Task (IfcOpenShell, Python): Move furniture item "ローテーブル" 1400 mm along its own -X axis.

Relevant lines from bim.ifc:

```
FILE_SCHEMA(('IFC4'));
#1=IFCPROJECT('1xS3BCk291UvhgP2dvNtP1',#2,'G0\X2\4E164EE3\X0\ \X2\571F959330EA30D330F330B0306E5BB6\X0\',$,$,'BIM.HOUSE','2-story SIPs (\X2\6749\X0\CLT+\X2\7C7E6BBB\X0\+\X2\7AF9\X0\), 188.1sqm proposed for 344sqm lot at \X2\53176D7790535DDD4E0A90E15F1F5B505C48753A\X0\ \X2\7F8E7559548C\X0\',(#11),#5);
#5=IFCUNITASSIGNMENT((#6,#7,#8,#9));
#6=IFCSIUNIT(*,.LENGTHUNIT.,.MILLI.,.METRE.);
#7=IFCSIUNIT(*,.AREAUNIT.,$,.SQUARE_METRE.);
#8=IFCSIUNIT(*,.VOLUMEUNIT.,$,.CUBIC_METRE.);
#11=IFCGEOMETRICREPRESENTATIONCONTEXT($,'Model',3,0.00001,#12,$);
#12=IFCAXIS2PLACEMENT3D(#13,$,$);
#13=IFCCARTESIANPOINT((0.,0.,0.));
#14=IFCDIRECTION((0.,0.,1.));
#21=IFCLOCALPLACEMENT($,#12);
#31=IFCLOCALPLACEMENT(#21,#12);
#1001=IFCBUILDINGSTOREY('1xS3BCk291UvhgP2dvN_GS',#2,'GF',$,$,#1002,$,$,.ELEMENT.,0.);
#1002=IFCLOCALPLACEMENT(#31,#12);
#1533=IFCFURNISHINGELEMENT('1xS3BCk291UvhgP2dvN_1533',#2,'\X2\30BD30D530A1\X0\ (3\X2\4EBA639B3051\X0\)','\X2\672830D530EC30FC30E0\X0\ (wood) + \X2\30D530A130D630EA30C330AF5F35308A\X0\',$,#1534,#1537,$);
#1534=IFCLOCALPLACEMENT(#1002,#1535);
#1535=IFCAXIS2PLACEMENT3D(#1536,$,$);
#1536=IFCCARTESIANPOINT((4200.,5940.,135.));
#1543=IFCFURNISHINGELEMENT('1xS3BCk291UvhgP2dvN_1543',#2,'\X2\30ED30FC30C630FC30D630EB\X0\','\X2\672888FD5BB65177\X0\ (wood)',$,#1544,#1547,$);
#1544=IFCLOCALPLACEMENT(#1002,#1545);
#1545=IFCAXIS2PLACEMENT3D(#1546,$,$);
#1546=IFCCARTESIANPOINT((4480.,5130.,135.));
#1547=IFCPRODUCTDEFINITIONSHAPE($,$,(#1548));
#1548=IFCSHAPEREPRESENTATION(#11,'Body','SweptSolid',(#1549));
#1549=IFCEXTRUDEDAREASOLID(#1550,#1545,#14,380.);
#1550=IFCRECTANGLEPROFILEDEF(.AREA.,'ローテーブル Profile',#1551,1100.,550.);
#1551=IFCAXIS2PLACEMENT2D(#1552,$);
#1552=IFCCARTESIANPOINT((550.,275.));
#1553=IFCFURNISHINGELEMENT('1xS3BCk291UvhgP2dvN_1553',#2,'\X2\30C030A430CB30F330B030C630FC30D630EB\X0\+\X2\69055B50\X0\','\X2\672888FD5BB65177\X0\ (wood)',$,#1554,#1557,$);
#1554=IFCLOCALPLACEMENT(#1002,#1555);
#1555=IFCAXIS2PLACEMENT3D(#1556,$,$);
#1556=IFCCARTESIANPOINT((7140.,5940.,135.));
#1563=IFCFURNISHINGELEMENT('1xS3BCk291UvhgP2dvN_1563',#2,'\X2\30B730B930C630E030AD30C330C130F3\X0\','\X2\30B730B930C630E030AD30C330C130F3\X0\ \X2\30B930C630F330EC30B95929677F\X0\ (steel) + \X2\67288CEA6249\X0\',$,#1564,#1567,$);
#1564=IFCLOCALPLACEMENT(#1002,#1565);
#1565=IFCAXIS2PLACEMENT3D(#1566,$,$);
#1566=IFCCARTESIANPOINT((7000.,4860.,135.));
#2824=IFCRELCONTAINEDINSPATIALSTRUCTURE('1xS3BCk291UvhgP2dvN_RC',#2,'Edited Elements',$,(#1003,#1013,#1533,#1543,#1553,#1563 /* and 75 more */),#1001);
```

```python
import ifcopenshell
import ifcopenshell.api.geometry
import ifcopenshell.util.placement

model = ifcopenshell.open("bim.ifc")

item = model.by_id(1543)
matrix = ifcopenshell.util.placement.get_local_placement(item.ObjectPlacement)
matrix[:3, 3] -= matrix[:3, 0] * 1400.0
ifcopenshell.api.geometry.edit_object_placement(model, product=item, matrix=matrix, is_si=False)

print(ifcopenshell.util.placement.get_local_placement(item.ObjectPlacement).round(3) + 0.0)

model.write("bim-out.ifc")
```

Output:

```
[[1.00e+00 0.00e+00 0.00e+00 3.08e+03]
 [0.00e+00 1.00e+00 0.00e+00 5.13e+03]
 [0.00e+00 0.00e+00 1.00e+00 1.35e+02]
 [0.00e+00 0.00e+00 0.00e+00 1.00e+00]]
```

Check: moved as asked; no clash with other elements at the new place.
